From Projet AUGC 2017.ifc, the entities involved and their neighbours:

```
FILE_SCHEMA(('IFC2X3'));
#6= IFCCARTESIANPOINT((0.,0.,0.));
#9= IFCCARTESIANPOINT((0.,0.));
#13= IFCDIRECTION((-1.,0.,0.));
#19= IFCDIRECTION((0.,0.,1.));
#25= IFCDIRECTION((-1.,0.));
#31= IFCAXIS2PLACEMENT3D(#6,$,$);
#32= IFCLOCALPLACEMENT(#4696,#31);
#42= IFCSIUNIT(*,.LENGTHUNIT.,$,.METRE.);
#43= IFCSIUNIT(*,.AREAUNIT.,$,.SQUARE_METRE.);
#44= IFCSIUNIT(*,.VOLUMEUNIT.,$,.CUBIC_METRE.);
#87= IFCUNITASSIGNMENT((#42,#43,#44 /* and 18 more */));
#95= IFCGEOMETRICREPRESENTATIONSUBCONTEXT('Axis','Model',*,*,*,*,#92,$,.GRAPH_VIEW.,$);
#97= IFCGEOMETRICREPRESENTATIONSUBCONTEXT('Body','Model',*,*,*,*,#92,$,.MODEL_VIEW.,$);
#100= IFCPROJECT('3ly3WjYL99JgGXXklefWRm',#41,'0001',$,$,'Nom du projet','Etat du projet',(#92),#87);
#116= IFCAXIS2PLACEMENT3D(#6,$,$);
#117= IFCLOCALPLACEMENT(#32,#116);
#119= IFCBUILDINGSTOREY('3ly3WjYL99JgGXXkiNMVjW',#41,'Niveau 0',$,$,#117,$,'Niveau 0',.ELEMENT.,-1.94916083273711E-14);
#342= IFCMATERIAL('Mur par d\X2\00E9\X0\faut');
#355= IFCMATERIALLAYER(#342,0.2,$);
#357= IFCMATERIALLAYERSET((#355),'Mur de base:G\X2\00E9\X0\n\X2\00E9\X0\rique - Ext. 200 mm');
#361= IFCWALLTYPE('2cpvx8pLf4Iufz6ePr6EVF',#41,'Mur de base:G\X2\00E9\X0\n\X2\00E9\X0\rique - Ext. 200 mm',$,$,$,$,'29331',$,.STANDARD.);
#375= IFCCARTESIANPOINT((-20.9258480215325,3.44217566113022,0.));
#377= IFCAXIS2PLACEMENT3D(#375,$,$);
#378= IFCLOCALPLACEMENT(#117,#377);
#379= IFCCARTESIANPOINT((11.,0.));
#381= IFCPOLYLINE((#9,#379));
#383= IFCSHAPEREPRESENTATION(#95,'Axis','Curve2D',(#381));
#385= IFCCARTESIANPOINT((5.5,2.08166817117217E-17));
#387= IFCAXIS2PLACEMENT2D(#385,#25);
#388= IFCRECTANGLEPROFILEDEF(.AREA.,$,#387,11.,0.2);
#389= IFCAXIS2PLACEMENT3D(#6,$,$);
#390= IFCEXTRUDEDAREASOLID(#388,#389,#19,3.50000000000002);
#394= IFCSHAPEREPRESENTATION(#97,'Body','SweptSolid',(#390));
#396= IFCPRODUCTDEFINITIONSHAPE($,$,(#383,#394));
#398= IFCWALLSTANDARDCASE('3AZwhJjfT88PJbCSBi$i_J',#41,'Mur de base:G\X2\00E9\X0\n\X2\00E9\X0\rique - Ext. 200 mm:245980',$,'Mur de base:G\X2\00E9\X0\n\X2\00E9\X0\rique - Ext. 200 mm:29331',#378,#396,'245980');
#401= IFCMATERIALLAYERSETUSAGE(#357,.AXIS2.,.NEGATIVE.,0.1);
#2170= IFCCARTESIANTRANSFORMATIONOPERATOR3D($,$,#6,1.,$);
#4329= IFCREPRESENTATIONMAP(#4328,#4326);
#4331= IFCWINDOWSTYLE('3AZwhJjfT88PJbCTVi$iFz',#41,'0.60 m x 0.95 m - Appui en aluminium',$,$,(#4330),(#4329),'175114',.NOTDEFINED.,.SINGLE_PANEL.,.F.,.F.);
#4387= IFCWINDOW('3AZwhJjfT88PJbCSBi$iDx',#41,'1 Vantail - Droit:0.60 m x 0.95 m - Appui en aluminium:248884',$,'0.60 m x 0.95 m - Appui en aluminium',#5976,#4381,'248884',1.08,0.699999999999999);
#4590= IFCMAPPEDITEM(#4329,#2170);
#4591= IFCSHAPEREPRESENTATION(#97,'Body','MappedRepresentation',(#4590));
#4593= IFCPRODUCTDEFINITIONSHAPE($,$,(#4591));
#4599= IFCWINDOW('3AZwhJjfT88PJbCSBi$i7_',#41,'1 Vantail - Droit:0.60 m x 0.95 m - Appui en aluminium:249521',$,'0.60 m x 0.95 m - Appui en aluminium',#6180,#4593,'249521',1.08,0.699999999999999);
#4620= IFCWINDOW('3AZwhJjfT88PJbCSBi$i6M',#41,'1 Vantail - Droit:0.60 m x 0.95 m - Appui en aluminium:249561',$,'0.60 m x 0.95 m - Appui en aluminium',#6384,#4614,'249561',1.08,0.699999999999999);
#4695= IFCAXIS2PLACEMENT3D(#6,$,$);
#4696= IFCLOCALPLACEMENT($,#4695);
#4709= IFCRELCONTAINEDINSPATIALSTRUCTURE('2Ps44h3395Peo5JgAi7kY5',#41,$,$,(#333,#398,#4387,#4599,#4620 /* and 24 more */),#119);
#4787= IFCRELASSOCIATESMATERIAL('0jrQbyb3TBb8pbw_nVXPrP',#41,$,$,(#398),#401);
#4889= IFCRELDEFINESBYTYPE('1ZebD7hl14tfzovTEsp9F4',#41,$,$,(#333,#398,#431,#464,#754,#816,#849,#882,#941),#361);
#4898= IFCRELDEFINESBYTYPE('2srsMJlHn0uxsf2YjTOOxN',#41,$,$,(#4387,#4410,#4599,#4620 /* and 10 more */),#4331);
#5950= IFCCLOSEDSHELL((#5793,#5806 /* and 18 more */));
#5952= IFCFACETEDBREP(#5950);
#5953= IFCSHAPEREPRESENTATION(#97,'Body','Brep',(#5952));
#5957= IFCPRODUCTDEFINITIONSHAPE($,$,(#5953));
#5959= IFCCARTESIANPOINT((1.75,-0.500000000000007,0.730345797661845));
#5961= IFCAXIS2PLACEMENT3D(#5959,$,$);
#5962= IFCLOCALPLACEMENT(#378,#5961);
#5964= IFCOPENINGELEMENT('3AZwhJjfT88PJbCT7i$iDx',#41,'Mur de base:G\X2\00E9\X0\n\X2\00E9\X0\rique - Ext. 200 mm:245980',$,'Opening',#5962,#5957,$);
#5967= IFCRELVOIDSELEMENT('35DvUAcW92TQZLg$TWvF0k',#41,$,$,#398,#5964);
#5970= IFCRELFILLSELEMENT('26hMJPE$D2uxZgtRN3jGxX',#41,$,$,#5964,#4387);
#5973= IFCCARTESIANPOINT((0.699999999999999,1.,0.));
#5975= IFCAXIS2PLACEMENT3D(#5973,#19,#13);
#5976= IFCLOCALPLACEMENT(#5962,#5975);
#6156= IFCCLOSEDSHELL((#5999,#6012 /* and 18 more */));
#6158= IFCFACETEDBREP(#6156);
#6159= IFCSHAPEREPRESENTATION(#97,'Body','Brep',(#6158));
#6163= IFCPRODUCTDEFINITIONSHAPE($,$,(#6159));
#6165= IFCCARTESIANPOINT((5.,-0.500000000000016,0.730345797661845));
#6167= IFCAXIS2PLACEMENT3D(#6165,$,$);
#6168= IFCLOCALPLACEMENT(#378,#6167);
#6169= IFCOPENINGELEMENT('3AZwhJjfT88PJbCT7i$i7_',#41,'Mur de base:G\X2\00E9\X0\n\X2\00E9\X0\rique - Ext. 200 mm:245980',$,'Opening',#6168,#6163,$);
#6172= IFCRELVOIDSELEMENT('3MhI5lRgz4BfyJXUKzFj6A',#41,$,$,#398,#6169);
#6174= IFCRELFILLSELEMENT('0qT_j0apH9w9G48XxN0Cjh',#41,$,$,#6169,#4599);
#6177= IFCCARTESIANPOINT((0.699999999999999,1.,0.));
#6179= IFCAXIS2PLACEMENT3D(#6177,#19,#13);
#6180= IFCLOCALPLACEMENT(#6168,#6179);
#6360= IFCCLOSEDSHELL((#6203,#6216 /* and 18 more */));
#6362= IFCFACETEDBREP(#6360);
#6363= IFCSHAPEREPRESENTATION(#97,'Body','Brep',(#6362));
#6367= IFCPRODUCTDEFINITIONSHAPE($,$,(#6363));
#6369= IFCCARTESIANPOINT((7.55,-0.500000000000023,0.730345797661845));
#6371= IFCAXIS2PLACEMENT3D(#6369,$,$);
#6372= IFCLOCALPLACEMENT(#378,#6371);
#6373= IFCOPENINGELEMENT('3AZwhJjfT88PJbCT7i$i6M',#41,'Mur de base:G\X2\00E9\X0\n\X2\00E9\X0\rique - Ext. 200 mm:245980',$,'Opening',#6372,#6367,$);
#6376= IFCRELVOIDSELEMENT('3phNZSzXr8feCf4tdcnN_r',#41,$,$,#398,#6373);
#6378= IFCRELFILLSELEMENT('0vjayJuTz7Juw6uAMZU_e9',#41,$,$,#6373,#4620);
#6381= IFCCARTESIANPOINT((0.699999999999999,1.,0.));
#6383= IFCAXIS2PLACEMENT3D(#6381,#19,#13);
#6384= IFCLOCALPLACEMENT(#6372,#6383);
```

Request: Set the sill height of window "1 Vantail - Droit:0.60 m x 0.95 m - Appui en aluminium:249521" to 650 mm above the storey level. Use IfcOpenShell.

```python
import numpy as np
import ifcopenshell
import ifcopenshell.api.geometry
import ifcopenshell.geom
import ifcopenshell.util.element
import ifcopenshell.util.placement
import ifcopenshell.util.shape
import ifcopenshell.util.unit

model = ifcopenshell.open("Projet AUGC 2017.ifc")
unit_scale = ifcopenshell.util.unit.calculate_unit_scale(model)

window = model.by_guid("3AZwhJjfT88PJbCSBi$i7_")
opening = window.FillsVoids[0].RelatingOpeningElement
storey = ifcopenshell.util.element.get_container(window, ifc_class="IfcBuildingStorey")
level = ifcopenshell.util.placement.get_local_placement(storey.ObjectPlacement)[2, 3]

# The opening's origin need not be at the sill, so measure its lowest point.
shape = ifcopenshell.geom.create_shape(ifcopenshell.geom.settings(), opening)
bottom = ifcopenshell.util.shape.get_shape_bottom_elevation(shape, shape.geometry) / unit_scale
dz = level + 0.65 / unit_scale - bottom

shift = np.array([0.0, 0.0, dz])
# The window is placed relative to its opening, so it follows when the opening moves.
matrix = ifcopenshell.util.placement.get_local_placement(opening.ObjectPlacement)
matrix[:3, 3] += shift
ifcopenshell.api.geometry.edit_object_placement(
    model, product=opening, matrix=matrix, is_si=False, should_transform_children=True
)

print(f"moved by {dz * unit_scale:+.3f} m")

model.write("Projet AUGC 2017_edited.ifc")
```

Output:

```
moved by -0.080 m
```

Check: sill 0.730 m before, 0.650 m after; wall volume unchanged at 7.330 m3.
